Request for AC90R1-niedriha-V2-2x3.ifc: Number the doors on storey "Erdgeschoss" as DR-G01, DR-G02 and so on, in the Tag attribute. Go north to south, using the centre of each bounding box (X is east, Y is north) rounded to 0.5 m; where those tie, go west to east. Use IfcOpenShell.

First a look at what the model holds.

```python
import ifcopenshell
import ifcopenshell.util.element
import ifcopenshell.util.placement

model = ifcopenshell.open("AC90R1-niedriha-V2-2x3.ifc")
print(model.schema)
storey = next(s for s in model.by_type("IfcBuildingStorey") if s.Name == "Erdgeschoss")
doors = [e for e in ifcopenshell.util.element.get_decomposition(storey) if e.is_a("IfcDoor")]
for e in sorted(doors, key=lambda e: e.id()):
    origin = ifcopenshell.util.placement.get_local_placement(e.ObjectPlacement)[:3, 3]
    print(e.id(), e.Tag, e.Name, origin.round(2) + 0.0, sep=" | ")
```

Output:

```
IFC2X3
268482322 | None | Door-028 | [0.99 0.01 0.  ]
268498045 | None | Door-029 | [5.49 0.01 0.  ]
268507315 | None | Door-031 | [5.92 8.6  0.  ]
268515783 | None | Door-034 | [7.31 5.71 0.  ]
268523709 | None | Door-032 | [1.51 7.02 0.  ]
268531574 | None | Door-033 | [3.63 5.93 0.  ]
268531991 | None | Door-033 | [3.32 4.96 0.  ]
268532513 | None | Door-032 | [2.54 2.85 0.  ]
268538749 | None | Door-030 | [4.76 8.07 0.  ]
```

```python
import ifcopenshell
import ifcopenshell.geom
import ifcopenshell.util.element
import ifcopenshell.util.shape

model = ifcopenshell.open("AC90R1-niedriha-V2-2x3.ifc")
settings = ifcopenshell.geom.settings()
settings.set("use-world-coords", True)


def centre(element):
    shape = ifcopenshell.geom.create_shape(settings, element)
    return ifcopenshell.util.shape.get_bbox_centroid(shape.geometry)


storey = next(s for s in model.by_type("IfcBuildingStorey") if s.Name == "Erdgeschoss")
doors = [e for e in ifcopenshell.util.element.get_decomposition(storey) if e.is_a("IfcDoor")]

# Insertion points can sit at a corner or the storey origin, so sort by the geometry (in metres).
centres = {e: centre(e) for e in doors}
doors.sort(key=lambda e: (-round(centres[e][1] / 0.5), centres[e][0]))

for i, e in enumerate(doors, start=1):
    number = f"DR-G{i:02d}"
    e.Tag = number
    print(e.id(), number)

model.write("AC90R1-niedriha-V2-2x3_edited.ifc")
```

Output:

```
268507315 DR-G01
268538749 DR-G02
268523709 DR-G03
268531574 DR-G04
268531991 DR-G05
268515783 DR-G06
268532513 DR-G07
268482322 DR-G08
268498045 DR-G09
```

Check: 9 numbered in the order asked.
